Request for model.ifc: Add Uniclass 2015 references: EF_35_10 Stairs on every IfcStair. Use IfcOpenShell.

First a look at what the model holds.

```python
import ifcopenshell

model = ifcopenshell.open("model.ifc")
print(model.schema)
print("classifications:", [c.Name for c in model.by_type("IfcClassification")])
for ifc_class in ("IfcDoor", "IfcRoof", "IfcStair", "IfcWall", "IfcWindow"):
    print(ifc_class, len(model.by_type(ifc_class)))
```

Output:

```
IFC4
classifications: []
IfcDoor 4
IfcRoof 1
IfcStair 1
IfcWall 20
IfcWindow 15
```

```python
import ifcopenshell
import ifcopenshell.api.classification

model = ifcopenshell.open("model.ifc")

system = ifcopenshell.api.classification.add_classification(model, classification="Uniclass 2015")

codes = {
    "IfcStair": ("EF_35_10", "Stairs"),
}
for ifc_class, (code, name) in codes.items():
    products = model.by_type(ifc_class)
    ifcopenshell.api.classification.add_reference(
        model, products=products, classification=system, identification=code, name=name
    )
    print(code, len(products))

model.write("model_v2.ifc")
```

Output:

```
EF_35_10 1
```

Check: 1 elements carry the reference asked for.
